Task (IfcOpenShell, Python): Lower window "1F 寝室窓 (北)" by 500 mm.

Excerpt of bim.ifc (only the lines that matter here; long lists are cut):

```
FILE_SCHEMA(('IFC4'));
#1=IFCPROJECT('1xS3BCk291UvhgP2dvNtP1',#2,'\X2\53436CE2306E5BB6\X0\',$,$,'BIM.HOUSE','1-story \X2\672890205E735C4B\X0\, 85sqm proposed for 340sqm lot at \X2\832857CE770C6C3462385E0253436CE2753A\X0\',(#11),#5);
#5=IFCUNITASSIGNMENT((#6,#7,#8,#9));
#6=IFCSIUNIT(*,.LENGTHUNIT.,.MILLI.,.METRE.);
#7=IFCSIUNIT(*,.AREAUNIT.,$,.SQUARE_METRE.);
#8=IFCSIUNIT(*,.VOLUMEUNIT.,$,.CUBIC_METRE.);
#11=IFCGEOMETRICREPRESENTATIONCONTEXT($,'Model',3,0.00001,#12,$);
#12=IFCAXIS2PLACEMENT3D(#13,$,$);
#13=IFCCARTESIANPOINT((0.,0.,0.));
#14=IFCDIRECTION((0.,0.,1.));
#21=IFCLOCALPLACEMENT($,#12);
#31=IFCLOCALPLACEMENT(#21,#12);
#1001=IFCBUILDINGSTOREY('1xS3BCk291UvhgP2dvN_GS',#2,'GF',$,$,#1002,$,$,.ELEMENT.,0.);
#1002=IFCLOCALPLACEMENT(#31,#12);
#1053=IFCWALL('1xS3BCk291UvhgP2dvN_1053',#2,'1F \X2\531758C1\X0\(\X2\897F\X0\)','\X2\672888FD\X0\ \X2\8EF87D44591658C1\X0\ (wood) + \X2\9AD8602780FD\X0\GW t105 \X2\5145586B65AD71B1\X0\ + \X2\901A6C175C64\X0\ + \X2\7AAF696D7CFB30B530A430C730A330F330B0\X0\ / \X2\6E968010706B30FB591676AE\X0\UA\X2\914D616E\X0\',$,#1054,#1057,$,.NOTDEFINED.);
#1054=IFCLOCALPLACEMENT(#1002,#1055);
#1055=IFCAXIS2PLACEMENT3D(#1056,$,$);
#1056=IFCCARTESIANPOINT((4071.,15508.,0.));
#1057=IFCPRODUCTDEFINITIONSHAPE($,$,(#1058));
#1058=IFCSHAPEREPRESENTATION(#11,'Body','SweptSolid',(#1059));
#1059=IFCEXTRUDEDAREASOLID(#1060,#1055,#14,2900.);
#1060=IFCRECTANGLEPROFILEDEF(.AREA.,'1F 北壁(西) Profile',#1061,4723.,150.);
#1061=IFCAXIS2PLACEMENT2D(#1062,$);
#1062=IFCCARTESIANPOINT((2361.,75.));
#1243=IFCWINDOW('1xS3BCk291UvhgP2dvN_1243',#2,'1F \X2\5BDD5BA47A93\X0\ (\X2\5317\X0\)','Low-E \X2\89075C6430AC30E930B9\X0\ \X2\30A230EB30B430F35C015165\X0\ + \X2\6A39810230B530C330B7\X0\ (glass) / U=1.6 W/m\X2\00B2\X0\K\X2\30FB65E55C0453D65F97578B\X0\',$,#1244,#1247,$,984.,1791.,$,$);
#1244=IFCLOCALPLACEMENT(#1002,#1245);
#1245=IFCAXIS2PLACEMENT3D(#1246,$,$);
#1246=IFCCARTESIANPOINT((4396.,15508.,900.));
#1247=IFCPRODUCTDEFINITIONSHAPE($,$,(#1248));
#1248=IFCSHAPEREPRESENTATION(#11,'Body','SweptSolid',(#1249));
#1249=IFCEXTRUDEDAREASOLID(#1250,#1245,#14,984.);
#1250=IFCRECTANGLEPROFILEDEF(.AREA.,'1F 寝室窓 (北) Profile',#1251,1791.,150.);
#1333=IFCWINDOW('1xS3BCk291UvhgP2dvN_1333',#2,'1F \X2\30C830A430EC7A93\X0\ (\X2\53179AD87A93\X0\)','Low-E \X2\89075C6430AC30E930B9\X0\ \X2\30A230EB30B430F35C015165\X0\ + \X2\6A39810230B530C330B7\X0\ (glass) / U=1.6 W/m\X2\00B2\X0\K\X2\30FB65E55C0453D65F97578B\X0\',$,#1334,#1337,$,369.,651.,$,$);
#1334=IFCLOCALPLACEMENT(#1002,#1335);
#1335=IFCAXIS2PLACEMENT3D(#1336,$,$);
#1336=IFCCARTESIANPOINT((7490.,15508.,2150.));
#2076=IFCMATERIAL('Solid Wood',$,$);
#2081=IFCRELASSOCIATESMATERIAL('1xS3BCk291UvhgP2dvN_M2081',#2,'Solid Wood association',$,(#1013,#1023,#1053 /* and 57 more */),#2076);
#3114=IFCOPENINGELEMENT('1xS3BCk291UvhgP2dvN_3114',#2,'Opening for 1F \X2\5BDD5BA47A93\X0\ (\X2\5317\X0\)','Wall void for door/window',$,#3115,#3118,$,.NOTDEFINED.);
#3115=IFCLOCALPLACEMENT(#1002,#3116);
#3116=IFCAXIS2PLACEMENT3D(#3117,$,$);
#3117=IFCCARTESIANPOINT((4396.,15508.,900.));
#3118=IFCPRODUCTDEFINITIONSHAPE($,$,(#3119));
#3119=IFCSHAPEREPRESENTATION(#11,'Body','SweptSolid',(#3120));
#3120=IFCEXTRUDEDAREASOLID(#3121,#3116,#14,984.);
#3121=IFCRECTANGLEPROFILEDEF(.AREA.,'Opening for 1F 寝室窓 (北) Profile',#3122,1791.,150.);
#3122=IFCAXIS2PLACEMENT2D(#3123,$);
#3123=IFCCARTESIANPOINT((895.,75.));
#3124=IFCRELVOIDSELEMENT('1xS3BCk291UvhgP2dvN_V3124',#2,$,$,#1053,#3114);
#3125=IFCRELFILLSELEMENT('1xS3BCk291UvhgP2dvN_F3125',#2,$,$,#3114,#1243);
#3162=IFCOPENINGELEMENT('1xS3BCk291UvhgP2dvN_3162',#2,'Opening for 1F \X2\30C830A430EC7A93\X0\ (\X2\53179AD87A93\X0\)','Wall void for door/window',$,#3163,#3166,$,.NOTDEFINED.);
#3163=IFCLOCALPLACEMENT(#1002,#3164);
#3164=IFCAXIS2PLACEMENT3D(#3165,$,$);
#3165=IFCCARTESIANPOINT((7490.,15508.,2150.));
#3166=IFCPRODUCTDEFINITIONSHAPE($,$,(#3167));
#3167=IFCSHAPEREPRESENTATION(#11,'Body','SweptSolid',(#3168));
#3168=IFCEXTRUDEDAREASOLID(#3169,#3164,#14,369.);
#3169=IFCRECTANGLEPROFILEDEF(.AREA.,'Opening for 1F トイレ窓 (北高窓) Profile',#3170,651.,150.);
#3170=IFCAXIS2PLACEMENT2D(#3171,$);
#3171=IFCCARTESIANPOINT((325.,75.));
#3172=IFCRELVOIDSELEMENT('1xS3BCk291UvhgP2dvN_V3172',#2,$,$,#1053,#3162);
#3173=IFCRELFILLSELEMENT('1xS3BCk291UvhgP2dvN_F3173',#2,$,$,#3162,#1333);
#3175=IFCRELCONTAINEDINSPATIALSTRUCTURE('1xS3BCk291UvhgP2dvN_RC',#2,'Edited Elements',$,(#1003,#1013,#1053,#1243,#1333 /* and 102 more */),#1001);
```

```python
import numpy as np
import ifcopenshell
import ifcopenshell.api.geometry
import ifcopenshell.util.placement
import ifcopenshell.util.unit

model = ifcopenshell.open("bim.ifc")
unit_scale = ifcopenshell.util.unit.calculate_unit_scale(model)

window = model.by_guid("1xS3BCk291UvhgP2dvN_1243")
opening = window.FillsVoids[0].RelatingOpeningElement
dz = -0.5 / unit_scale

shift = np.array([0.0, 0.0, dz])
# The window is not placed relative to its opening, so move both.
for product in (opening, window):
    matrix = ifcopenshell.util.placement.get_local_placement(product.ObjectPlacement)
    matrix[:3, 3] += shift
    ifcopenshell.api.geometry.edit_object_placement(model, product=product, matrix=matrix, is_si=False)

print(f"moved by {dz * unit_scale:+.3f} m")

model.write("bim_rev.ifc")
```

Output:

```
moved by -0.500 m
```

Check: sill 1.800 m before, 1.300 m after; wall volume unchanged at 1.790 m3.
